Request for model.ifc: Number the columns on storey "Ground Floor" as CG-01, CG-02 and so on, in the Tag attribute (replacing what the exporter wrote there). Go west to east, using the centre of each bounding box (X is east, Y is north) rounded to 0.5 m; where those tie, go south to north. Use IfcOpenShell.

First a look at what the model holds.

```python
import ifcopenshell
import ifcopenshell.util.element
import ifcopenshell.util.placement

model = ifcopenshell.open("model.ifc")
print(model.schema)
storey = next(s for s in model.by_type("IfcBuildingStorey") if s.Name == "Ground Floor")
columns = [e for e in ifcopenshell.util.element.get_decomposition(storey) if e.is_a("IfcColumn")]
for e in sorted(columns, key=lambda e: e.id()):
    origin = ifcopenshell.util.placement.get_local_placement(e.ObjectPlacement)[:3, 3]
    print(e.id(), e.Tag, e.Name, origin.round(2) + 0.0, sep=" | ")
```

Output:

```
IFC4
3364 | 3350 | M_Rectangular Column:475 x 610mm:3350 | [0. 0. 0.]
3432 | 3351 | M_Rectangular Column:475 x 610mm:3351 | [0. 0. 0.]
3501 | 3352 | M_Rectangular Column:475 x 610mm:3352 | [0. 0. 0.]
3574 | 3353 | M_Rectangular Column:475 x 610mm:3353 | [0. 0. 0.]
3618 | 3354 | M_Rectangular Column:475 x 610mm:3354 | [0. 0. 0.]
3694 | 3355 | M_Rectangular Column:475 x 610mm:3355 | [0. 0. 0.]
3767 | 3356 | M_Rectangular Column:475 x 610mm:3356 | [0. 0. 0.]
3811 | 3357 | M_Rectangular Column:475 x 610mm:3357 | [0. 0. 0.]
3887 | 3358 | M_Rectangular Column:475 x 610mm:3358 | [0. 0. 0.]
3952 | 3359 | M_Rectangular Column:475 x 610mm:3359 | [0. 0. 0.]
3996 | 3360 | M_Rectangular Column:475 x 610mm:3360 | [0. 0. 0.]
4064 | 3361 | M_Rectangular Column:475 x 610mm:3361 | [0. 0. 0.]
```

```python
import ifcopenshell
import ifcopenshell.geom
import ifcopenshell.util.element
import ifcopenshell.util.shape

model = ifcopenshell.open("model.ifc")
settings = ifcopenshell.geom.settings()
settings.set("use-world-coords", True)


def centre(element):
    shape = ifcopenshell.geom.create_shape(settings, element)
    return ifcopenshell.util.shape.get_bbox_centroid(shape.geometry)


storey = next(s for s in model.by_type("IfcBuildingStorey") if s.Name == "Ground Floor")
columns = [e for e in ifcopenshell.util.element.get_decomposition(storey) if e.is_a("IfcColumn")]

# Insertion points can sit at a corner or the storey origin, so sort by the geometry (in metres).
centres = {e: centre(e) for e in columns}
columns.sort(key=lambda e: (round(centres[e][0] / 0.5), centres[e][1]))

for i, e in enumerate(columns, start=1):
    number = f"CG-{i:02d}"
    e.Tag = number
    print(e.id(), number)

model.write("model_edited.ifc")
```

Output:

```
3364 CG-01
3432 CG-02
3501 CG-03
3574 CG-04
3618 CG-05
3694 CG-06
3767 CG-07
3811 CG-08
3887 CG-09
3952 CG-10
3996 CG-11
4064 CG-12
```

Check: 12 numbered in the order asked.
